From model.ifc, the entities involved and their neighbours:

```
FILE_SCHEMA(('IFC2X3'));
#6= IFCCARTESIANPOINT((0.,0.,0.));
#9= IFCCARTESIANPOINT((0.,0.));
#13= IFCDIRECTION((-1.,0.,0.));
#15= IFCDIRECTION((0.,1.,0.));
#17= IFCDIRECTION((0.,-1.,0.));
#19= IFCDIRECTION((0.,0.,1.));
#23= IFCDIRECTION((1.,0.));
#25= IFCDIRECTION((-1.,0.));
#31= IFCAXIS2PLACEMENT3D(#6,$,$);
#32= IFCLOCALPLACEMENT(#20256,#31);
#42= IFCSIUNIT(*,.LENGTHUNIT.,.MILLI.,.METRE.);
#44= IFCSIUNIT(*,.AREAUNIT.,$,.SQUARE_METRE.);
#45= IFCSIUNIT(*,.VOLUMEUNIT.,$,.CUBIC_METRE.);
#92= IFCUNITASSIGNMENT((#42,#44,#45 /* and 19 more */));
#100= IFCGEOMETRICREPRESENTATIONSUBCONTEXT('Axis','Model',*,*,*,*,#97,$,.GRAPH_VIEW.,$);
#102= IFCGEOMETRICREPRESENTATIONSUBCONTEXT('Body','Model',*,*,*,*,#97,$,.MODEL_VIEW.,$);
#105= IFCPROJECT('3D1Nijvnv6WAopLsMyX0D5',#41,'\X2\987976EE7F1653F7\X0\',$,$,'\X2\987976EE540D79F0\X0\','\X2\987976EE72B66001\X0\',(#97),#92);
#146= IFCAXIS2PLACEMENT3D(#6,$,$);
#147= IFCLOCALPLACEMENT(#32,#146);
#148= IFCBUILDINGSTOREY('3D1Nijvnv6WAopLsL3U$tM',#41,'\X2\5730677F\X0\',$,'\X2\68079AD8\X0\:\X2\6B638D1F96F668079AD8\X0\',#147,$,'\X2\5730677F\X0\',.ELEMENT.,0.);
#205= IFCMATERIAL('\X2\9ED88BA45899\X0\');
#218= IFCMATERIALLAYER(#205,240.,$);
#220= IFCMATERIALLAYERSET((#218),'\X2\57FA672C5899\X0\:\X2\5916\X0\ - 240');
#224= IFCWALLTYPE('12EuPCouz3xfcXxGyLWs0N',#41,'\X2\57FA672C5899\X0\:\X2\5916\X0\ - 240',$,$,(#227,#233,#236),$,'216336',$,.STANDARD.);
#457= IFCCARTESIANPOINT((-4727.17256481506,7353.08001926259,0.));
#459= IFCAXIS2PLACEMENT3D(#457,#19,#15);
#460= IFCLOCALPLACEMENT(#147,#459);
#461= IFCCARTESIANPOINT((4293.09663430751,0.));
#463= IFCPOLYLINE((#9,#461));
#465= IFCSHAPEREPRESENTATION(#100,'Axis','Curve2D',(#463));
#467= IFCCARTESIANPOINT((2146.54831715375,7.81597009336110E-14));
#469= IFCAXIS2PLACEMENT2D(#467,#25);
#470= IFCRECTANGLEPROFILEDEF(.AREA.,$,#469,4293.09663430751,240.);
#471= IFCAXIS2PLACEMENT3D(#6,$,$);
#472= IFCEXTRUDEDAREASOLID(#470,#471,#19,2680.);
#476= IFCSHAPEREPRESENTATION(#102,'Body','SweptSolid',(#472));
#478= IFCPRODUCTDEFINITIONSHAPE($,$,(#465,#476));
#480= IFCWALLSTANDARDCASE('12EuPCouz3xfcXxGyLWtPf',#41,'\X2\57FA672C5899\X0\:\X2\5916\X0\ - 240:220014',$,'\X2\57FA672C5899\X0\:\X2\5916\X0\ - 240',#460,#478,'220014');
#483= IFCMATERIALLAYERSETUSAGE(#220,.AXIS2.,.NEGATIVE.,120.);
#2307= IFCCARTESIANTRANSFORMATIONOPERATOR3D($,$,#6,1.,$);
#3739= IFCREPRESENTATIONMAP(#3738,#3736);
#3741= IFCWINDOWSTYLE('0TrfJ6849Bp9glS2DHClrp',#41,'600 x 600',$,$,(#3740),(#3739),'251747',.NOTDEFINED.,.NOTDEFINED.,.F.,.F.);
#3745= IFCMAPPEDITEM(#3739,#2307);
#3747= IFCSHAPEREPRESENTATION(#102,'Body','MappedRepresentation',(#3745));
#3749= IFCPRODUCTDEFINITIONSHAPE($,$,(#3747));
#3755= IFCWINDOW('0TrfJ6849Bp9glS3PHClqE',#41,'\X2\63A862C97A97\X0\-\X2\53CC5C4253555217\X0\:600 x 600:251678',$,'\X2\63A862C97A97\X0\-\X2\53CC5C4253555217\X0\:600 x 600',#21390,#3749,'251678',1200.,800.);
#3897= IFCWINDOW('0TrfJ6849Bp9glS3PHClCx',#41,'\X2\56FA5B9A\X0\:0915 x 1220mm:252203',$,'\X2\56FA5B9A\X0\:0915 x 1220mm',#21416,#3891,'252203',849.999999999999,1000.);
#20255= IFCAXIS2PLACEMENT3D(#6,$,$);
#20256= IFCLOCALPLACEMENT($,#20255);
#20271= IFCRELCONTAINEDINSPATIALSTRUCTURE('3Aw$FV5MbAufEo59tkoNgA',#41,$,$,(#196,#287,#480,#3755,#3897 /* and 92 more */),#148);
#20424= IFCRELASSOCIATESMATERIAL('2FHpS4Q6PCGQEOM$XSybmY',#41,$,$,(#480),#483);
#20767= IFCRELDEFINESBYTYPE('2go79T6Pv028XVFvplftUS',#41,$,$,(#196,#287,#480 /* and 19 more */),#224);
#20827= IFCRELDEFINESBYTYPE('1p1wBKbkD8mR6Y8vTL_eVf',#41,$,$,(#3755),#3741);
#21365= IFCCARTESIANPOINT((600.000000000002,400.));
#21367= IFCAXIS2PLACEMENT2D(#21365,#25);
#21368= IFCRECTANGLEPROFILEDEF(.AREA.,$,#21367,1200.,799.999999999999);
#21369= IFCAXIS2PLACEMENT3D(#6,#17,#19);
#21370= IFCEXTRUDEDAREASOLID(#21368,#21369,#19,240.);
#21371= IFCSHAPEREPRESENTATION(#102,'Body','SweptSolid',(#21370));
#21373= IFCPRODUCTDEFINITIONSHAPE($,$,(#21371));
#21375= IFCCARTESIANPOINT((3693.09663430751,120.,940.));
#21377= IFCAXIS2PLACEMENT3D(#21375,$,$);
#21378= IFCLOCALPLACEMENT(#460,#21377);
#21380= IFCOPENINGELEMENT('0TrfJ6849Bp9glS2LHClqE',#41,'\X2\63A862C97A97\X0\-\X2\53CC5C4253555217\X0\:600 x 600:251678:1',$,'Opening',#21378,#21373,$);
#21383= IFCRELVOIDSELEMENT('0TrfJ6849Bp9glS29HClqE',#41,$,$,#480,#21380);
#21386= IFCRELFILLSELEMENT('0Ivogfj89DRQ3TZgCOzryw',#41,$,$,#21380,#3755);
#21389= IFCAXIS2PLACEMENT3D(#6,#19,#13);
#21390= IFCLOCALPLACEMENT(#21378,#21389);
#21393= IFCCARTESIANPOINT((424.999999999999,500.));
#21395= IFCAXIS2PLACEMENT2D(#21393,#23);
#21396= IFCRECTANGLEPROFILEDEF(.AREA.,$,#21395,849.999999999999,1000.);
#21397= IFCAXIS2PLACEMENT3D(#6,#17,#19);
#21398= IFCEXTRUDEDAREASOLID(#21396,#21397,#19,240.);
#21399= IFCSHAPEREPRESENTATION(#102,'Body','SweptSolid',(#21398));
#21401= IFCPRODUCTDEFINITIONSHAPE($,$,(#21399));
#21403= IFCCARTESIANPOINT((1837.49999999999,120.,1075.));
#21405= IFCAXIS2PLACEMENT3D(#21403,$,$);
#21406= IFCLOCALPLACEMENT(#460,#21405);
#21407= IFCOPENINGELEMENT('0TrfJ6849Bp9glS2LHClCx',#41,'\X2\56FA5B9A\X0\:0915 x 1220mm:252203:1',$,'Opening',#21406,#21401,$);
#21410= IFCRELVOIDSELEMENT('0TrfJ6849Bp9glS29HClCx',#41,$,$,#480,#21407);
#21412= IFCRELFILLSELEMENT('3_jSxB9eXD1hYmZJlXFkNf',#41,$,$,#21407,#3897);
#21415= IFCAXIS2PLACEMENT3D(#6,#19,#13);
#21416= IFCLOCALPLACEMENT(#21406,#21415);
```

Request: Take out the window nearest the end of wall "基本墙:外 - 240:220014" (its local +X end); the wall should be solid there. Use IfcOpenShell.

```python
import ifcopenshell
import ifcopenshell.api.feature
import ifcopenshell.api.root
import ifcopenshell.geom
import ifcopenshell.util.shape

model = ifcopenshell.open("model.ifc")
settings = ifcopenshell.geom.settings()


def volume(element):
    """Net volume in cubic metres, openings subtracted."""
    shape = ifcopenshell.geom.create_shape(settings, element)
    return ifcopenshell.util.shape.get_volume(shape.geometry)


window = model.by_id(3755)
opening = window.FillsVoids[0].RelatingOpeningElement
wall = opening.VoidsElements[0].RelatingBuildingElement
before = volume(wall)

ifcopenshell.api.root.remove_product(model, product=window)
ifcopenshell.api.feature.remove_feature(model, feature=opening)

after = volume(wall)

print(f"wall volume {before:.3f} -> {after:.3f} m3")

model.write("model_edited.ifc")
```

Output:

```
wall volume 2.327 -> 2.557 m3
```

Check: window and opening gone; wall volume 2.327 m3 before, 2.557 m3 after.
